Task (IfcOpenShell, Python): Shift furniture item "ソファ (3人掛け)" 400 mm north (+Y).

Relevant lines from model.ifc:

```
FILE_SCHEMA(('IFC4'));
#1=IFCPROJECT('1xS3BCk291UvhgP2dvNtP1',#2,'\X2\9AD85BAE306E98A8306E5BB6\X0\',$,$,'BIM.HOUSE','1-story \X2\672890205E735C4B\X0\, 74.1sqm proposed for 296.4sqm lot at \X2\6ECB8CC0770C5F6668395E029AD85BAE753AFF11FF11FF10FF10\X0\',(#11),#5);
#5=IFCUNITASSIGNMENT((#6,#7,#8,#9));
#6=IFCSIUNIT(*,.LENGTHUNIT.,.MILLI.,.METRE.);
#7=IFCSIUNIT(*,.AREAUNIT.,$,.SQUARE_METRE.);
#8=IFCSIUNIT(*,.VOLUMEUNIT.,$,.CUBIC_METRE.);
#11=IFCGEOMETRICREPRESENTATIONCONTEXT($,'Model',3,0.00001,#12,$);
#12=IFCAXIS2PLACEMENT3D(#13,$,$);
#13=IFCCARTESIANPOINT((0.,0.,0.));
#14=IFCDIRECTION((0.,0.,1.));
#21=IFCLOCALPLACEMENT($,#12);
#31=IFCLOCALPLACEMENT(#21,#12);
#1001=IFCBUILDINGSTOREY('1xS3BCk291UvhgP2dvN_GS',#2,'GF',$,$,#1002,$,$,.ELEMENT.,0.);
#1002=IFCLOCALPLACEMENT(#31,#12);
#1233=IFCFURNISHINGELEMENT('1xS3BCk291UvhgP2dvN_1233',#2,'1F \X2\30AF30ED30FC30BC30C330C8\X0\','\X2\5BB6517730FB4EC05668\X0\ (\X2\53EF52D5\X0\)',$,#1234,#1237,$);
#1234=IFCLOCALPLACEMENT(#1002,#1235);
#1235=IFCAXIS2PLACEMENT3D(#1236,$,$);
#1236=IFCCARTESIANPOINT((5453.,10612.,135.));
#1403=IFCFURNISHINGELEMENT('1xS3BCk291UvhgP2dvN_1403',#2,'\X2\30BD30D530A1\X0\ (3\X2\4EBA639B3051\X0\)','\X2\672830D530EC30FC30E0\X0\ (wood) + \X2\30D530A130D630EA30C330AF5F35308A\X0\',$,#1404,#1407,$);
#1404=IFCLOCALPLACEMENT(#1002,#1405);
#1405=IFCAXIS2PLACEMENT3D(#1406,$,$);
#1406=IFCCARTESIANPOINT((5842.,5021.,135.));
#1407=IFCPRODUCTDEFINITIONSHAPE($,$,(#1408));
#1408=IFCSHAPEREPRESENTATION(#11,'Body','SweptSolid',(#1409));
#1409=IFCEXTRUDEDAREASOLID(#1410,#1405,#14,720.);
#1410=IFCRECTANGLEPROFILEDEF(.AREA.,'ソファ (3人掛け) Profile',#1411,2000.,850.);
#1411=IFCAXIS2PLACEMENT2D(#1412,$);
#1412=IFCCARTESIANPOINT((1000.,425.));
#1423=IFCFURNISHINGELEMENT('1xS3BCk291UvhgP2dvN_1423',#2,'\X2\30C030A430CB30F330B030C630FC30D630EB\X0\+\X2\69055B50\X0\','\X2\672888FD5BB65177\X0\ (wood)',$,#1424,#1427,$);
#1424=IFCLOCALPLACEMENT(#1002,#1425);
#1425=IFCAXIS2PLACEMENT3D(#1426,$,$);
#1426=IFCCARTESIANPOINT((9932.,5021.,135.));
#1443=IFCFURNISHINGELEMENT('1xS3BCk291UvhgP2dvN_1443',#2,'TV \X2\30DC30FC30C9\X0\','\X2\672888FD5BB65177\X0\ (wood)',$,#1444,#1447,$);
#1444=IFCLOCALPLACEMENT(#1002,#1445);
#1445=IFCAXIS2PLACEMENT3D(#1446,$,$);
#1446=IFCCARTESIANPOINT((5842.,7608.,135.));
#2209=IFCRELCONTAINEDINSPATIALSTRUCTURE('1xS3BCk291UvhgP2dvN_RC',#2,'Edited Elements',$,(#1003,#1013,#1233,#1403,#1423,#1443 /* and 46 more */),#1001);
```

```python
import ifcopenshell
import ifcopenshell.api.geometry
import ifcopenshell.util.placement
import ifcopenshell.util.unit

model = ifcopenshell.open("model.ifc")
unit_scale = ifcopenshell.util.unit.calculate_unit_scale(model)

item = model.by_guid("1xS3BCk291UvhgP2dvN_1403")
matrix = ifcopenshell.util.placement.get_local_placement(item.ObjectPlacement)
matrix[1, 3] += 0.4 / unit_scale
ifcopenshell.api.geometry.edit_object_placement(model, product=item, matrix=matrix, is_si=False)

print(ifcopenshell.util.placement.get_local_placement(item.ObjectPlacement).round(3) + 0.0)

model.write("model_edited.ifc")
```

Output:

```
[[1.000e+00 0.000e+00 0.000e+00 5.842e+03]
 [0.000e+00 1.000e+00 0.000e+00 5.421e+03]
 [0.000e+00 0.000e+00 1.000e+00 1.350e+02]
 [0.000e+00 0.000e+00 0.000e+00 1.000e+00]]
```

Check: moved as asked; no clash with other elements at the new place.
